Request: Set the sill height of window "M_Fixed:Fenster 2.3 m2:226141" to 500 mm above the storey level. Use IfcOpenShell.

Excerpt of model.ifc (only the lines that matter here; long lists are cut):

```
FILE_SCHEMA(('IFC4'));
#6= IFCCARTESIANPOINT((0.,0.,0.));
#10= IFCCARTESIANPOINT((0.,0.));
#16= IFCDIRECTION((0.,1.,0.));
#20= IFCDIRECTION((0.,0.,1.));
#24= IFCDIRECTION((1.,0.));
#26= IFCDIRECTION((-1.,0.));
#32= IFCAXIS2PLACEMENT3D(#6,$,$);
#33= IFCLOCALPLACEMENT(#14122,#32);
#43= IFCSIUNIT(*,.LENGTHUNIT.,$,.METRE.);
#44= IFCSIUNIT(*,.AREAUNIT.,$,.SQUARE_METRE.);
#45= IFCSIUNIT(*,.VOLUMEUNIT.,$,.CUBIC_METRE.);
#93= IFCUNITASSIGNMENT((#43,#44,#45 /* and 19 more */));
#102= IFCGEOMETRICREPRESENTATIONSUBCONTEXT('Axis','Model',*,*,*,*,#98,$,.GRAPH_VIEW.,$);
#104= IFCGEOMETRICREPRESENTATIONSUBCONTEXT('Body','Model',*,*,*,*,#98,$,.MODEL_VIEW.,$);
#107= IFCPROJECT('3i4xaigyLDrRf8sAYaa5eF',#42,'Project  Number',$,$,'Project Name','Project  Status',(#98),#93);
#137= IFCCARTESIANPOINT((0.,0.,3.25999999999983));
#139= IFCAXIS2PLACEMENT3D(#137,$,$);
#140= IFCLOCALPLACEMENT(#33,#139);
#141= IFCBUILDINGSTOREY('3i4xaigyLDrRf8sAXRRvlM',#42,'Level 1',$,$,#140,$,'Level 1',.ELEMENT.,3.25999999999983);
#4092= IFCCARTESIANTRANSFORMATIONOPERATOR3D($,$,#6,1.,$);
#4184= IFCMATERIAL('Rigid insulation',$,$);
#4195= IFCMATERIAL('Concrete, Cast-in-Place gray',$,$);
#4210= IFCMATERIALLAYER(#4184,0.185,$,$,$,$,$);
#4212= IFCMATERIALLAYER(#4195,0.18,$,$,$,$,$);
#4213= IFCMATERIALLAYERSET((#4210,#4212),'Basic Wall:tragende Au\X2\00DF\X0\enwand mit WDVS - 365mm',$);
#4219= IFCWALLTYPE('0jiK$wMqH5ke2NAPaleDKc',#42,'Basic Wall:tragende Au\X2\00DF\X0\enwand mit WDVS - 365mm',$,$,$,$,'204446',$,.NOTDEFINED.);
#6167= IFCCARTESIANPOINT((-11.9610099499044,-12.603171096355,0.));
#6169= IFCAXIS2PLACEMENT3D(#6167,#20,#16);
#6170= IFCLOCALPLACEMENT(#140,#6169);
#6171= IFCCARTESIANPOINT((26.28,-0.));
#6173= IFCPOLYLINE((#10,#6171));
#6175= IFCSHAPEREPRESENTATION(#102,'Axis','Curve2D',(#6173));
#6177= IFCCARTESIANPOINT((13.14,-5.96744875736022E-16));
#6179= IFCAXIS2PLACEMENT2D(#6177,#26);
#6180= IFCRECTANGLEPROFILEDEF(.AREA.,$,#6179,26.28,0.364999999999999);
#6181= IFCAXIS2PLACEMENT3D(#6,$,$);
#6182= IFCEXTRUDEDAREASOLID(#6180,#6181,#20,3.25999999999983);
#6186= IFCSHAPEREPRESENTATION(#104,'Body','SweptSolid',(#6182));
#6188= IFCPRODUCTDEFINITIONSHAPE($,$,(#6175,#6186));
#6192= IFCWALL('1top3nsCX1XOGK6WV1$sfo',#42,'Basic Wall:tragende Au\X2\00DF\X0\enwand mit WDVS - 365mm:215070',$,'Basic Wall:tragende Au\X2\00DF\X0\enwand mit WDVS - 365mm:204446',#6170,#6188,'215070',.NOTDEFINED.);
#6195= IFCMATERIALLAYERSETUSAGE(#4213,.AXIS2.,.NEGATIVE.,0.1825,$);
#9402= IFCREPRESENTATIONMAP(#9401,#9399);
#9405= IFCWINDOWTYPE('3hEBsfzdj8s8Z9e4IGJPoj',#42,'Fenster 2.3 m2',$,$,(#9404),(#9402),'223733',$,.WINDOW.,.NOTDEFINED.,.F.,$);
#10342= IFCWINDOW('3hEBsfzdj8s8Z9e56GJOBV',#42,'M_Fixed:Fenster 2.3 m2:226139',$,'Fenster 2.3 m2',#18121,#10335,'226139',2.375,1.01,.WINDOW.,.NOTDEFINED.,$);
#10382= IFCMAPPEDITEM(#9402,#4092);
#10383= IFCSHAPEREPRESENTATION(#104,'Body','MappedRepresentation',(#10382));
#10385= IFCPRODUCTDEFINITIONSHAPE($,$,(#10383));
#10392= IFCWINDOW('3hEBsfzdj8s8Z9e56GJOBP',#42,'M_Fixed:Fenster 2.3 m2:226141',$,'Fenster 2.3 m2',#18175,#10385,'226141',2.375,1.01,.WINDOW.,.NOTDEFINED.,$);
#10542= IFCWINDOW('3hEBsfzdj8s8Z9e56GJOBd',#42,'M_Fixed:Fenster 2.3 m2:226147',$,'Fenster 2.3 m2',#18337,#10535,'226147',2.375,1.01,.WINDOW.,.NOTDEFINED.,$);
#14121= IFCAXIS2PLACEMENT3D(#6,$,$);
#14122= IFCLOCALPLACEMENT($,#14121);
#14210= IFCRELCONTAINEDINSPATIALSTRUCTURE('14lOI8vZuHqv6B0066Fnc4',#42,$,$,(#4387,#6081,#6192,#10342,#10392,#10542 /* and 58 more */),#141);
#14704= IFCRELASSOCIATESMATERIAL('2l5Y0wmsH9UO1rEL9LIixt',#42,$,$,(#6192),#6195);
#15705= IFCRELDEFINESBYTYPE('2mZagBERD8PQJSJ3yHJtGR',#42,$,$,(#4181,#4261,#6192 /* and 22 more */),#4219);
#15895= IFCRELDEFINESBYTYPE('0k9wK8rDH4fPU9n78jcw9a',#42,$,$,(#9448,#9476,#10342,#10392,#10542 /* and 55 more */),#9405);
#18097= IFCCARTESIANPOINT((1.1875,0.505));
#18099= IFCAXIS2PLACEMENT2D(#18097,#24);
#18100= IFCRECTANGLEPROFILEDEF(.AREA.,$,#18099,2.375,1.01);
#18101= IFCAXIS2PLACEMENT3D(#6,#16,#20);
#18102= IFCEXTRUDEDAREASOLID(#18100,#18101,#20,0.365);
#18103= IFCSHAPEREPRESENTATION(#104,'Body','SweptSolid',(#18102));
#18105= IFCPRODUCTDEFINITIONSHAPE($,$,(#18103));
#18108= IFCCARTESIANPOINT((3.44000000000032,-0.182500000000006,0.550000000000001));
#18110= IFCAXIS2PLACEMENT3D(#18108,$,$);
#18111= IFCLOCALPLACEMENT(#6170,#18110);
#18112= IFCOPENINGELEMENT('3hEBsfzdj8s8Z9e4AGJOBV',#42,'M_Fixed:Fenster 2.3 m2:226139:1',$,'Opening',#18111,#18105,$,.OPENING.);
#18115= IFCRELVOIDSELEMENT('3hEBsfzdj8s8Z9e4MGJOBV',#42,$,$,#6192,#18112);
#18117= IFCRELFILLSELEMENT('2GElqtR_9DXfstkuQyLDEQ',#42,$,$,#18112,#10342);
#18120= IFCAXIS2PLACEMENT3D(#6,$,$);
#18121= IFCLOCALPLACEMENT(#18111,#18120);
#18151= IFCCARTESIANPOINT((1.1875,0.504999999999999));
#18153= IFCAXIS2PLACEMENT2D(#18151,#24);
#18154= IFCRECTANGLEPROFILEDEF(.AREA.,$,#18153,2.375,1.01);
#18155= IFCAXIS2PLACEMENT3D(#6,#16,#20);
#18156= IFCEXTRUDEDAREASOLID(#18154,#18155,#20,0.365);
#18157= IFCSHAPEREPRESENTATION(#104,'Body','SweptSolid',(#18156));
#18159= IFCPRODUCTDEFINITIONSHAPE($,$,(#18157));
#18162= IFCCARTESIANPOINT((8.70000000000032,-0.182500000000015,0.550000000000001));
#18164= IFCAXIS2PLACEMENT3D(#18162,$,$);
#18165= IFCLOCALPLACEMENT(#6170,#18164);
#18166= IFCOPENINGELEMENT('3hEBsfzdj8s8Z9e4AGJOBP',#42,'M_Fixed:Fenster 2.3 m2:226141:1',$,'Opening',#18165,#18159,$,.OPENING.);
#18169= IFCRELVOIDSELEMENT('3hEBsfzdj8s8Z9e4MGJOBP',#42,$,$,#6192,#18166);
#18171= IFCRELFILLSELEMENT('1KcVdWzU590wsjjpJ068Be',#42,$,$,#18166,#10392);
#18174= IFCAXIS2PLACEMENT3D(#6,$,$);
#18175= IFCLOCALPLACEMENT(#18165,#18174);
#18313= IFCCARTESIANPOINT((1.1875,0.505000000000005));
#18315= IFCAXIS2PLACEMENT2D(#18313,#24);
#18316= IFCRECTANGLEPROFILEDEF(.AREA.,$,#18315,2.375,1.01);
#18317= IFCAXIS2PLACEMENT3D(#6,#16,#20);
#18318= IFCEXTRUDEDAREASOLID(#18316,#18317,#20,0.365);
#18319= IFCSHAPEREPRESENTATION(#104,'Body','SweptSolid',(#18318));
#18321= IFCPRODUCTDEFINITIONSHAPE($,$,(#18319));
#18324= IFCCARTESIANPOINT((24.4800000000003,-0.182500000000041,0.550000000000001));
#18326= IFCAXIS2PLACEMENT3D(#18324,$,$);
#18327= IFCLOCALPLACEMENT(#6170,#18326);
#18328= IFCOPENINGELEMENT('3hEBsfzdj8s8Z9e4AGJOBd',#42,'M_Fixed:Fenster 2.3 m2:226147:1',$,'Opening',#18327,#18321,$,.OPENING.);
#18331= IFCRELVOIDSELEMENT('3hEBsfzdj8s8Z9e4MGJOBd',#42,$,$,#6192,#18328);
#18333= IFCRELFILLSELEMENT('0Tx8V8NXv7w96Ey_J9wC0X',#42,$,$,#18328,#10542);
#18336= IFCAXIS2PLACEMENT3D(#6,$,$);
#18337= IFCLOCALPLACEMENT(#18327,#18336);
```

```python
import numpy as np
import ifcopenshell
import ifcopenshell.api.geometry
import ifcopenshell.geom
import ifcopenshell.util.element
import ifcopenshell.util.placement
import ifcopenshell.util.shape
import ifcopenshell.util.unit

model = ifcopenshell.open("model.ifc")
unit_scale = ifcopenshell.util.unit.calculate_unit_scale(model)

window = model.by_guid("3hEBsfzdj8s8Z9e56GJOBP")
opening = window.FillsVoids[0].RelatingOpeningElement
storey = ifcopenshell.util.element.get_container(window, ifc_class="IfcBuildingStorey")
level = ifcopenshell.util.placement.get_local_placement(storey.ObjectPlacement)[2, 3]

# The opening's origin need not be at the sill, so measure its lowest point.
shape = ifcopenshell.geom.create_shape(ifcopenshell.geom.settings(), opening)
bottom = ifcopenshell.util.shape.get_shape_bottom_elevation(shape, shape.geometry) / unit_scale
dz = level + 0.5 - bottom

shift = np.array([0.0, 0.0, dz])
# The window is placed relative to its opening, so it follows when the opening moves.
matrix = ifcopenshell.util.placement.get_local_placement(opening.ObjectPlacement)
matrix[:3, 3] += shift
ifcopenshell.api.geometry.edit_object_placement(
    model, product=opening, matrix=matrix, is_si=False, should_transform_children=True
)

print(f"moved by {dz * unit_scale:+.3f} m")

model.write("model_updated.ifc")
```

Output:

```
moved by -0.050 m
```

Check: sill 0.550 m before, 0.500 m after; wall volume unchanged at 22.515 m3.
